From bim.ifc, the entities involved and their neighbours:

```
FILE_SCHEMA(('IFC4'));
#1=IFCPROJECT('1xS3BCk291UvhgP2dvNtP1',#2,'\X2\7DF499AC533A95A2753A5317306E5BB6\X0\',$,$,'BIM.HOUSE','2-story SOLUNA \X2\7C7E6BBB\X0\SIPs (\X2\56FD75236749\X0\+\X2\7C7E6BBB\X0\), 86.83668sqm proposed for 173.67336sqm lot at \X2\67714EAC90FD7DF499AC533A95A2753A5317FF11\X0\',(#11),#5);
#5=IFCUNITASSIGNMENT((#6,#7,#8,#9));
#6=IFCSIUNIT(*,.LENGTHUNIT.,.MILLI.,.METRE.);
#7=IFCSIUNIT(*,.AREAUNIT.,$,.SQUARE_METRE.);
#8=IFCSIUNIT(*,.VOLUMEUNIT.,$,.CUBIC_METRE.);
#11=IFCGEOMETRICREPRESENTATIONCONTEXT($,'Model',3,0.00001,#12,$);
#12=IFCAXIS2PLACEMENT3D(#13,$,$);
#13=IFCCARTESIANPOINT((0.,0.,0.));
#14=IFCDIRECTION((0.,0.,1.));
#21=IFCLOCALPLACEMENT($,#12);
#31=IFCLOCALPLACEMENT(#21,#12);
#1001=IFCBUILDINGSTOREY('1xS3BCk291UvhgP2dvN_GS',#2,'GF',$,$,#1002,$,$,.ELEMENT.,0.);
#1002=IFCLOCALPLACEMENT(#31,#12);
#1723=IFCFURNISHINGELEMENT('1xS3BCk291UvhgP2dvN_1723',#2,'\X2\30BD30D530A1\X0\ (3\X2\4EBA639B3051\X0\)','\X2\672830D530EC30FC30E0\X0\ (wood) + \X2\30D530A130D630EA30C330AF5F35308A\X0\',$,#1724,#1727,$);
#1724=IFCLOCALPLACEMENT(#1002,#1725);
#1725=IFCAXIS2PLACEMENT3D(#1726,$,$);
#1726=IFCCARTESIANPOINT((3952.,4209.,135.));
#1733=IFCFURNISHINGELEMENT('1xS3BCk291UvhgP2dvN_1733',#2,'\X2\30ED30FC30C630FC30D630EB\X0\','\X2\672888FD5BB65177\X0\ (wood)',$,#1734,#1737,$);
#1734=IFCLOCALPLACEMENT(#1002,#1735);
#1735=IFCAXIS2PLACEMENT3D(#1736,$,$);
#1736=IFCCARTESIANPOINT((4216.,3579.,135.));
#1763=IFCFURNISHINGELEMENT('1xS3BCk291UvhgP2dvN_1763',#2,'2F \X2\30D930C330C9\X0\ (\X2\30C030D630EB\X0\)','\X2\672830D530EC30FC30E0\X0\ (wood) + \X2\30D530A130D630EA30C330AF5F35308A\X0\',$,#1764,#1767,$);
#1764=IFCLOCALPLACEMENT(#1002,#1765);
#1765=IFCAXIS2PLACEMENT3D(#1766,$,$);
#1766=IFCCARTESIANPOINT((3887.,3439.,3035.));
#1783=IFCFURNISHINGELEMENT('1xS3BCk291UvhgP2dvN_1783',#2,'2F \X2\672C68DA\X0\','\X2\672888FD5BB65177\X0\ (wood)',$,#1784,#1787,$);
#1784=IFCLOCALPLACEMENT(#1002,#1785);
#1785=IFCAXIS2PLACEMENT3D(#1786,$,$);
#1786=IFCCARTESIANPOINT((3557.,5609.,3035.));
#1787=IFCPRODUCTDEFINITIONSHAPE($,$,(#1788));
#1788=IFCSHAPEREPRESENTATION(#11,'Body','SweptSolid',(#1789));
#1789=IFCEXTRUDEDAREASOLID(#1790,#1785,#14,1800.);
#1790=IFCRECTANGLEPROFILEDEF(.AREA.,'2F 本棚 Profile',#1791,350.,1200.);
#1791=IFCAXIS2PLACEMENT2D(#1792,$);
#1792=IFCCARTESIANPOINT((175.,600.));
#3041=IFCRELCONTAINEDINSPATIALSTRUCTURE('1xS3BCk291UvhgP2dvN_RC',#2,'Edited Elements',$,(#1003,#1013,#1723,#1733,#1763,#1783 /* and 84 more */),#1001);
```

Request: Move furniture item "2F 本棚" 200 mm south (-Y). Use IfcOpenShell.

```python
import ifcopenshell
import ifcopenshell.api.geometry
import ifcopenshell.util.placement
import ifcopenshell.util.unit

model = ifcopenshell.open("bim.ifc")
unit_scale = ifcopenshell.util.unit.calculate_unit_scale(model)

item = model.by_guid("1xS3BCk291UvhgP2dvN_1783")
matrix = ifcopenshell.util.placement.get_local_placement(item.ObjectPlacement)
matrix[1, 3] -= 0.2 / unit_scale
ifcopenshell.api.geometry.edit_object_placement(model, product=item, matrix=matrix, is_si=False)

print(ifcopenshell.util.placement.get_local_placement(item.ObjectPlacement).round(3) + 0.0)

model.write("bim-out.ifc")
```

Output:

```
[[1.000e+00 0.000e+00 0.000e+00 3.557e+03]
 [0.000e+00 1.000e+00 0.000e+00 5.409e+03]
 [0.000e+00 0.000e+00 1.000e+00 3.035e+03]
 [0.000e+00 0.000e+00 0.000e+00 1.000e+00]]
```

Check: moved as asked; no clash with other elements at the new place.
